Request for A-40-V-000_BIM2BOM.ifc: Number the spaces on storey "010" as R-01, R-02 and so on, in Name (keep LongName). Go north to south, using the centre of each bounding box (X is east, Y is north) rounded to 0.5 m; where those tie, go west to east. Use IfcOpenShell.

First a look at what the model holds.

```python
import ifcopenshell
import ifcopenshell.util.element
import ifcopenshell.util.placement

model = ifcopenshell.open("A-40-V-000_BIM2BOM.ifc")
print(model.schema)
storey = next(s for s in model.by_type("IfcBuildingStorey") if s.Name == "010")
spaces = [e for e in ifcopenshell.util.element.get_decomposition(storey) if e.is_a("IfcSpace")]
for e in sorted(spaces, key=lambda e: e.id()):
    origin = ifcopenshell.util.placement.get_local_placement(e.ObjectPlacement)[:3, 3]
    print(e.id(), e.Name, e.LongName, origin.round(2) + 0.0, sep=" | ")
```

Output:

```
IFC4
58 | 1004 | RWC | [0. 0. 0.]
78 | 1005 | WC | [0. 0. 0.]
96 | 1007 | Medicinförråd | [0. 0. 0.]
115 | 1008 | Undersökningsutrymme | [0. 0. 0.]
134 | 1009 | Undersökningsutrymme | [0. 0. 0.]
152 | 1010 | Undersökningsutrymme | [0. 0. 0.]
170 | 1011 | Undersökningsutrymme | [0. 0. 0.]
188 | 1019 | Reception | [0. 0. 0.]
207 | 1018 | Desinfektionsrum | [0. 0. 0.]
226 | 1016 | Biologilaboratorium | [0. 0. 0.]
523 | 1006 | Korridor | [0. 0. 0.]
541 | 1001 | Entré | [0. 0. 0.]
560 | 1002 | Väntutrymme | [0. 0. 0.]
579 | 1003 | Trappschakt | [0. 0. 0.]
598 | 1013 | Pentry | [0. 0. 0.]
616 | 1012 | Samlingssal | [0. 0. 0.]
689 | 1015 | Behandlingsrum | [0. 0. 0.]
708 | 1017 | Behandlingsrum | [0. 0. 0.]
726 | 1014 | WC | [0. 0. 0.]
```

```python
import ifcopenshell
import ifcopenshell.geom
import ifcopenshell.util.element
import ifcopenshell.util.shape

model = ifcopenshell.open("A-40-V-000_BIM2BOM.ifc")
settings = ifcopenshell.geom.settings()
settings.set("use-world-coords", True)


def centre(element):
    shape = ifcopenshell.geom.create_shape(settings, element)
    return ifcopenshell.util.shape.get_bbox_centroid(shape.geometry)


storey = next(s for s in model.by_type("IfcBuildingStorey") if s.Name == "010")
spaces = [e for e in ifcopenshell.util.element.get_decomposition(storey) if e.is_a("IfcSpace")]

# Insertion points can sit at a corner or the storey origin, so sort by the geometry (in metres).
centres = {e: centre(e) for e in spaces}
spaces.sort(key=lambda e: (-round(centres[e][1] / 0.5), centres[e][0]))

for i, e in enumerate(spaces, start=1):
    number = f"R-{i:02d}"
    e.Name = number
    print(e.id(), number)

model.write("A-40-V-000_BIM2BOM_v2.ifc")
```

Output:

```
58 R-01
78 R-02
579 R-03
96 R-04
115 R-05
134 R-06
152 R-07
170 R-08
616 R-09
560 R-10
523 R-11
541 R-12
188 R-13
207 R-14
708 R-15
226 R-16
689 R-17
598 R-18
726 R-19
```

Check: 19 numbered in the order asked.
